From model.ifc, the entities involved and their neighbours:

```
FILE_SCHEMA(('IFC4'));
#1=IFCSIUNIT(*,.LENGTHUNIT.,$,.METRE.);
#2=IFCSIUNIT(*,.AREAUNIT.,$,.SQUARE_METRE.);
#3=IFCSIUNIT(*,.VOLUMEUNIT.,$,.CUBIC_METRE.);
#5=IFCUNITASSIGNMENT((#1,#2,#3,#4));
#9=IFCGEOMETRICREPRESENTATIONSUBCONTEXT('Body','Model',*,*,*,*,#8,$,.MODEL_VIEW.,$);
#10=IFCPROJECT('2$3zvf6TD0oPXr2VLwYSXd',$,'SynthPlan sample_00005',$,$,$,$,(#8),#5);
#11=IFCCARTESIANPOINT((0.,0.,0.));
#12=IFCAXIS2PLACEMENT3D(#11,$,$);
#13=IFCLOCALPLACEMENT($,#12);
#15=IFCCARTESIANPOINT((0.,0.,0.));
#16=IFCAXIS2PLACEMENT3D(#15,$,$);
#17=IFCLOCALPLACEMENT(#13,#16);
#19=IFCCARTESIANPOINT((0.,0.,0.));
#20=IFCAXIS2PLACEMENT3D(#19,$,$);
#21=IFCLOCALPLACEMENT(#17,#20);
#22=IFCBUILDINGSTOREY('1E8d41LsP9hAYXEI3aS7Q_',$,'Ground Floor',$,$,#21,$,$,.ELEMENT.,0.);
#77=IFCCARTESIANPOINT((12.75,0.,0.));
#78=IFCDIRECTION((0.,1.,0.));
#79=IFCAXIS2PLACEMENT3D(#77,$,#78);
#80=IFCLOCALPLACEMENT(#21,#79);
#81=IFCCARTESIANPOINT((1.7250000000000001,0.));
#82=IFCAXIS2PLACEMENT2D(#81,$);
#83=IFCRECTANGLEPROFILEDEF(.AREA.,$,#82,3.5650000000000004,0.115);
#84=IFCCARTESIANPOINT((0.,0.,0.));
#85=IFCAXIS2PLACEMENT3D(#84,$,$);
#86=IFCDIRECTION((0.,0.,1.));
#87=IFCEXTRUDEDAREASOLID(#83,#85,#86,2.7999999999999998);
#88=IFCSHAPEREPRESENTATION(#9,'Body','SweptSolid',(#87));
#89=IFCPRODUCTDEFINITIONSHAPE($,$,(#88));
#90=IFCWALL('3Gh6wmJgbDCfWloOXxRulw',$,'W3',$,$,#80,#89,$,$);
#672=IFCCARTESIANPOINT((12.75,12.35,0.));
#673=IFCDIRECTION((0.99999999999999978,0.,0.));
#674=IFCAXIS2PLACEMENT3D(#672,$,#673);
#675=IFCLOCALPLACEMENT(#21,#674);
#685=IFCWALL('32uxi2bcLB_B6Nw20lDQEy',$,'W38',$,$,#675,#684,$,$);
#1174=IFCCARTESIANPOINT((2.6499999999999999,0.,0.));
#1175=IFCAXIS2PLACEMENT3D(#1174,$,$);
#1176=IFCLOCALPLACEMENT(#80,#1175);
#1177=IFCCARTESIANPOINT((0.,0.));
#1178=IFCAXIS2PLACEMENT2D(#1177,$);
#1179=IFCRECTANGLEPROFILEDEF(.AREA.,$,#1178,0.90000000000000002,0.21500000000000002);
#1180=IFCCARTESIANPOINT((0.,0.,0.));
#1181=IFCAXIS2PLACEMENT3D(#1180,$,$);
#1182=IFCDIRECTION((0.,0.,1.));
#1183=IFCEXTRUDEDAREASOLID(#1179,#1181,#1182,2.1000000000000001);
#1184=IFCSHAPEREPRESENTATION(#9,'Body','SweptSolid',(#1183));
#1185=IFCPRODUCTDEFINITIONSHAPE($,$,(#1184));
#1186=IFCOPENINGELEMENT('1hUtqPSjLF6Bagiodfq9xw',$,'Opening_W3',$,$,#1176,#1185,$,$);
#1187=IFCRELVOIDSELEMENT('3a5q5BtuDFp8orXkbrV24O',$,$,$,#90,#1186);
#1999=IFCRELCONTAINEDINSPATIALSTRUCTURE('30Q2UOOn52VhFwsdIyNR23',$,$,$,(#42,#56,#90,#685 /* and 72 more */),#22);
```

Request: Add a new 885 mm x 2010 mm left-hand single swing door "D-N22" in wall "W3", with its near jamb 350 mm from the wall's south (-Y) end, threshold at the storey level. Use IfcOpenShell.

```python
import numpy as np
import ifcopenshell
import ifcopenshell.api.feature
import ifcopenshell.api.geometry
import ifcopenshell.api.root
import ifcopenshell.api.spatial
import ifcopenshell.geom
import ifcopenshell.util.element
import ifcopenshell.util.placement
import ifcopenshell.util.representation
import ifcopenshell.util.shape
import ifcopenshell.util.unit

model = ifcopenshell.open("model.ifc")
unit_scale = ifcopenshell.util.unit.calculate_unit_scale(model)
settings = ifcopenshell.geom.settings()


def volume(element):
    """Net volume in cubic metres, openings subtracted."""
    shape = ifcopenshell.geom.create_shape(settings, element)
    return ifcopenshell.util.shape.get_volume(shape.geometry)


wall = model.by_id(90)
storey = ifcopenshell.util.element.get_container(wall, ifc_class="IfcBuildingStorey")
context = ifcopenshell.util.representation.get_context(model, "Model", "Body", "MODEL_VIEW")
before = volume(wall)

width, height, from_end, sill = 0.885, 2.01, 0.35, 0.0  # metres

# The wall runs along its own X axis, and the end named is its -X end.
wall_shape = ifcopenshell.geom.create_shape(settings, wall)
x, y, z = ifcopenshell.util.shape.get_vertices(wall_shape.geometry).T
start = x.min() + from_end
face, thickness = float(y.min()), float(y.max() - y.min())
wall_matrix = ifcopenshell.util.placement.get_local_placement(wall.ObjectPlacement)
level = ifcopenshell.util.placement.get_local_placement(storey.ObjectPlacement)[2, 3]


def in_wall(x, y):
    """Placement at x, y metres in the wall's axes, at sill height."""
    matrix = wall_matrix.copy()
    matrix[:, 3] = wall_matrix @ np.array([x / unit_scale, y / unit_scale, 0.0, 1.0])
    matrix[2, 3] = level + sill / unit_scale
    return matrix


# Opening: a box that overshoots both wall faces by 50 mm.
opening = ifcopenshell.api.root.create_entity(model, ifc_class="IfcOpeningElement", predefined_type="OPENING")
box = ifcopenshell.api.geometry.add_wall_representation(
    model, context=context, length=width, height=height, thickness=thickness + 0.1
)
ifcopenshell.api.geometry.assign_representation(model, product=opening, representation=box)
ifcopenshell.api.geometry.edit_object_placement(model, product=opening, matrix=in_wall(start, face - 0.05), is_si=False)
ifcopenshell.api.feature.add_feature(model, feature=opening, element=wall)

door = ifcopenshell.api.root.create_entity(model, ifc_class="IfcDoor", name="D-N22", predefined_type="DOOR")
door.OverallWidth, door.OverallHeight = width / unit_scale, height / unit_scale
door.OperationType = "SINGLE_SWING_LEFT"
body = ifcopenshell.api.geometry.add_door_representation(
    model,
    context=context,
    overall_width=door.OverallWidth,
    overall_height=door.OverallHeight,
    operation_type="SINGLE_SWING_LEFT",
    lining_properties={"LiningDepth": thickness / unit_scale, "ThresholdDepth": thickness / unit_scale},
)
ifcopenshell.api.geometry.assign_representation(model, product=door, representation=body)
ifcopenshell.api.spatial.assign_container(model, products=[door], relating_structure=storey)
ifcopenshell.api.feature.add_filling(model, opening=opening, element=door)

# The lining spans the wall, so the door starts at the wall face.
ifcopenshell.api.geometry.edit_object_placement(model, product=door, matrix=in_wall(start, face), is_si=False)

after = volume(wall)

print(f"wall volume {before:.3f} -> {after:.3f} m3")

model.write("model_edited.ifc")
```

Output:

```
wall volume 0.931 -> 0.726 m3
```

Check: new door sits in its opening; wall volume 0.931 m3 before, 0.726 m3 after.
